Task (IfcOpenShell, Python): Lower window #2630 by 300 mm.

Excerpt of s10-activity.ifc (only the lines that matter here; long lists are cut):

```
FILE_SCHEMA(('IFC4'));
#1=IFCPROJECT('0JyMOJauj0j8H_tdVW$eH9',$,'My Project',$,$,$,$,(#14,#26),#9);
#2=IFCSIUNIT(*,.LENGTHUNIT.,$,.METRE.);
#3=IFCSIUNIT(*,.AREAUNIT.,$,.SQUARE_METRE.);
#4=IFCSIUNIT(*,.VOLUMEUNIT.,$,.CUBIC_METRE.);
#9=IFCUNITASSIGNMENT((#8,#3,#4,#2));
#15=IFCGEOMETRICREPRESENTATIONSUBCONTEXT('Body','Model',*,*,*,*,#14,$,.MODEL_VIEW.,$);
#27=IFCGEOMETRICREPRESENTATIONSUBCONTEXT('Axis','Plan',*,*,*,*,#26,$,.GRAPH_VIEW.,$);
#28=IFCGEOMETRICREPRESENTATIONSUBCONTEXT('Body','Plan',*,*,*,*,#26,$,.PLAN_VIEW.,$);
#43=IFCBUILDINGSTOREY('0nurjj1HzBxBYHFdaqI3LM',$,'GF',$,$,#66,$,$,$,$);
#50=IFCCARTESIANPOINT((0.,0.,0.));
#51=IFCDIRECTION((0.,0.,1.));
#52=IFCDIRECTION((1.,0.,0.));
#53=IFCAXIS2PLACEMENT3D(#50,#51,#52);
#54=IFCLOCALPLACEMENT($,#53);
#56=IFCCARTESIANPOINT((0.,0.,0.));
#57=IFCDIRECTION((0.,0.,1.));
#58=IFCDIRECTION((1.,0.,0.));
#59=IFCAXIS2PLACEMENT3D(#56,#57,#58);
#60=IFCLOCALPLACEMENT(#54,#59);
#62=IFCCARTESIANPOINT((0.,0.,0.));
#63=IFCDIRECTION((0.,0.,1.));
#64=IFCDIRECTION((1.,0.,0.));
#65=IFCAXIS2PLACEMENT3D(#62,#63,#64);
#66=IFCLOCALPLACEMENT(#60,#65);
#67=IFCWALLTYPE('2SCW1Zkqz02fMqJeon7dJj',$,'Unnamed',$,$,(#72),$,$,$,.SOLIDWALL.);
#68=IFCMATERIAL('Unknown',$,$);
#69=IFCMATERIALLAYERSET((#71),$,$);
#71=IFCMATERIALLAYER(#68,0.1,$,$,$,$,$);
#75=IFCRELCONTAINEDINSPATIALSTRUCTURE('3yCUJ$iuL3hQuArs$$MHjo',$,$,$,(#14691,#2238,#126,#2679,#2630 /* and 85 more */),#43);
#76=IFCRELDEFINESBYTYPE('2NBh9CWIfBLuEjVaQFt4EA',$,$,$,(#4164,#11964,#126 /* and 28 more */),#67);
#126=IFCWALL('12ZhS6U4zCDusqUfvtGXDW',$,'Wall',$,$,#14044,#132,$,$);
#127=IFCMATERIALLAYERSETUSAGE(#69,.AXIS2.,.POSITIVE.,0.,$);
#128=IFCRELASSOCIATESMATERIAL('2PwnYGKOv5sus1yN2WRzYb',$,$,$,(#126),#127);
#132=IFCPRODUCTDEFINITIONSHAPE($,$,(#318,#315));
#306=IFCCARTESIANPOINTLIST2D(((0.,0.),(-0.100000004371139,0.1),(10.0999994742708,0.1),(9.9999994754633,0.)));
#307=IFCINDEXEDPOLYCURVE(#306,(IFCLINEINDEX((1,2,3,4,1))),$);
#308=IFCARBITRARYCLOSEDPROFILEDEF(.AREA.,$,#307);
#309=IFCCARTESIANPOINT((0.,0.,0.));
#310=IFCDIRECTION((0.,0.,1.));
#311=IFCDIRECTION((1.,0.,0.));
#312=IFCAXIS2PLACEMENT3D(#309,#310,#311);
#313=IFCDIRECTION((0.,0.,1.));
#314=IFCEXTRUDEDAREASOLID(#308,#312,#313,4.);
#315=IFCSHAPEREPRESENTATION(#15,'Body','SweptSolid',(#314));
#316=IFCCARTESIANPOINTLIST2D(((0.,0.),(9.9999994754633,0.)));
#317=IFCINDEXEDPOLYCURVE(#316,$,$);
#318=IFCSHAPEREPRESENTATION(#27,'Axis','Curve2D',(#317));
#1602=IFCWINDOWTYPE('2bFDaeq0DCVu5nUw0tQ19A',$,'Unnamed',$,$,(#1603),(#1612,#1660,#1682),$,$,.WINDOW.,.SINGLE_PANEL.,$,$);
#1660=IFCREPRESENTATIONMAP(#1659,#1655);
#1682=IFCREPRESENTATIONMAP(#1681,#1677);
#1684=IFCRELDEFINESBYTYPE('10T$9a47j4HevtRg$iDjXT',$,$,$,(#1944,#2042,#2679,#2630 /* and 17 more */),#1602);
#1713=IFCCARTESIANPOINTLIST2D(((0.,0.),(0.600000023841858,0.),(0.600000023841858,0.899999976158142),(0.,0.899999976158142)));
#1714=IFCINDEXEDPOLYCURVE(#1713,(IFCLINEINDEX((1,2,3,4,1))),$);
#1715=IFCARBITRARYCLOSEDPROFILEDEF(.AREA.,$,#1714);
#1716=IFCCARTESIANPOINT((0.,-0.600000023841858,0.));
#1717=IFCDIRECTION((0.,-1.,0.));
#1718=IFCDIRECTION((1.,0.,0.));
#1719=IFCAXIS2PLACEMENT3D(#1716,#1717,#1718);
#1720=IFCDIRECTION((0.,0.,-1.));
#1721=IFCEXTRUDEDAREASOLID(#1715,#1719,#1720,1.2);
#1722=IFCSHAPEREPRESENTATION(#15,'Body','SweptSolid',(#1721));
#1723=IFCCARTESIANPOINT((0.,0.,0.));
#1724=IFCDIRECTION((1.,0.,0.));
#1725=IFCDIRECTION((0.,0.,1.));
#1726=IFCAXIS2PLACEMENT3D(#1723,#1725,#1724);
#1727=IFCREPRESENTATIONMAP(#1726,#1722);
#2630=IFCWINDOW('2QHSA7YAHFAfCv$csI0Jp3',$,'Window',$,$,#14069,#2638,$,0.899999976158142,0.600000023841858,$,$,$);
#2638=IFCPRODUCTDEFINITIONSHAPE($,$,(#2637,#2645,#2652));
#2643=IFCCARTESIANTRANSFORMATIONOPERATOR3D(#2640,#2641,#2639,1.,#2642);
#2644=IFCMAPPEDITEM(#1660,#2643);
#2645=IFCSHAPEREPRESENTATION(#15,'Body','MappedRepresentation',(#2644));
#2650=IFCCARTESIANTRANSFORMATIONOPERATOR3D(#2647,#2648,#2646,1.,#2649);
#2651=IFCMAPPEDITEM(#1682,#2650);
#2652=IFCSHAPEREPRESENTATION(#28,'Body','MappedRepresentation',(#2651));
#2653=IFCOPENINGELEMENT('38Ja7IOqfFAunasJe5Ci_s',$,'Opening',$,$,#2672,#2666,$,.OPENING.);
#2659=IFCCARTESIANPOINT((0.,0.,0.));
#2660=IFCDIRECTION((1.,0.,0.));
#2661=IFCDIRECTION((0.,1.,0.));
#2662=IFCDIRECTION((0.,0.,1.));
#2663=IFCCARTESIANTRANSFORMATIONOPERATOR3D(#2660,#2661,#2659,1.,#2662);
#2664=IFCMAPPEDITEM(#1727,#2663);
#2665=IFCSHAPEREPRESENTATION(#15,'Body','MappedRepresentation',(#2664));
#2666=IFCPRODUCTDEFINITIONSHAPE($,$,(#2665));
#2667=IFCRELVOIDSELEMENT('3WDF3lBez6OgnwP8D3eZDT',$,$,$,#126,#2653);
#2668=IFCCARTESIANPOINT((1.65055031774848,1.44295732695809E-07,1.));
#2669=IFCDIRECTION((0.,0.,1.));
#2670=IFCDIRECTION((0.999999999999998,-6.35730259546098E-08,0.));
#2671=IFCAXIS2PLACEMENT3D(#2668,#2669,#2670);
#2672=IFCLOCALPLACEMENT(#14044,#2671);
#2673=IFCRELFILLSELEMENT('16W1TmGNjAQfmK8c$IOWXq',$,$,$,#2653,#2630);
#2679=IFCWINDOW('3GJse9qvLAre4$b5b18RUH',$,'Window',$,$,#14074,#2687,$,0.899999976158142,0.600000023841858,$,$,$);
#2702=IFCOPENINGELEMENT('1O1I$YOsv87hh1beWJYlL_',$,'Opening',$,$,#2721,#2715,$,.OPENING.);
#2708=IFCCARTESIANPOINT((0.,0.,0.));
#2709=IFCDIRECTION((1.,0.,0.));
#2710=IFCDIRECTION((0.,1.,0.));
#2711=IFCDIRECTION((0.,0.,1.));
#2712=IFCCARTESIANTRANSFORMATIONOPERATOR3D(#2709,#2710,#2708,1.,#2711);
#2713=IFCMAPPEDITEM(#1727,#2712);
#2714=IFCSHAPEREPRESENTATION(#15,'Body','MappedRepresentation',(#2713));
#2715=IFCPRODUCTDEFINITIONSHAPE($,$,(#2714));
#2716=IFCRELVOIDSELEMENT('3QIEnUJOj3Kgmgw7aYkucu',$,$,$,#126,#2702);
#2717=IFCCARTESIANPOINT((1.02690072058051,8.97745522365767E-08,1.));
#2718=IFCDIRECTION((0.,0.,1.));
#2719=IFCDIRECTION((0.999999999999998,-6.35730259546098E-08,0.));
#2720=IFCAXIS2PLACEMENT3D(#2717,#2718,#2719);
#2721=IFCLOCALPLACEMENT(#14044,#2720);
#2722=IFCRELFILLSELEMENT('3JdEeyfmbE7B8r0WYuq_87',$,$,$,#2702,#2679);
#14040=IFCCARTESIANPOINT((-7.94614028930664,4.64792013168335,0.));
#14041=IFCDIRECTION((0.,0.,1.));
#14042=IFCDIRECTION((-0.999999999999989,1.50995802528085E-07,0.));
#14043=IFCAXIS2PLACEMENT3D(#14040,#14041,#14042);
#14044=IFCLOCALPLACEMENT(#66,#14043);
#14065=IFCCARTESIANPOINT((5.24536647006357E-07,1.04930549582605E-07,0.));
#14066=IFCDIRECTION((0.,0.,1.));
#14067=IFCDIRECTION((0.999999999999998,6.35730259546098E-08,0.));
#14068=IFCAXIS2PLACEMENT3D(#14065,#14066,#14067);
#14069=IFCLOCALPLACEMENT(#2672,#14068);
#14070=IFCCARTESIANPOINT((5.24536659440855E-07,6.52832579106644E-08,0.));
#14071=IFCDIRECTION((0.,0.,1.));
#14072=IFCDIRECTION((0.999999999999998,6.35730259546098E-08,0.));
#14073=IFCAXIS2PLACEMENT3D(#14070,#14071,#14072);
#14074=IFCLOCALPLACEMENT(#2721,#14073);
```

```python
import numpy as np
import ifcopenshell
import ifcopenshell.api.geometry
import ifcopenshell.util.placement
import ifcopenshell.util.unit

model = ifcopenshell.open("s10-activity.ifc")
unit_scale = ifcopenshell.util.unit.calculate_unit_scale(model)

window = model.by_guid("2QHSA7YAHFAfCv$csI0Jp3")
opening = window.FillsVoids[0].RelatingOpeningElement
dz = -0.3 / unit_scale

shift = np.array([0.0, 0.0, dz])
# The window is placed relative to its opening, so it follows when the opening moves.
matrix = ifcopenshell.util.placement.get_local_placement(opening.ObjectPlacement)
matrix[:3, 3] += shift
ifcopenshell.api.geometry.edit_object_placement(
    model, product=opening, matrix=matrix, is_si=False, should_transform_children=True
)

print(f"moved by {dz * unit_scale:+.3f} m")

model.write("s10-activity_edited.ifc")
```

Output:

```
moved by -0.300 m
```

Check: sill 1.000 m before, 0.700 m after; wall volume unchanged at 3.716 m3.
